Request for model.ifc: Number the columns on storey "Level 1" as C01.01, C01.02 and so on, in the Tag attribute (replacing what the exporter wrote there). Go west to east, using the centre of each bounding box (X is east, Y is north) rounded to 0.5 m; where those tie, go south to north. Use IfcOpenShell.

First a look at what the model holds.

```python
import ifcopenshell
import ifcopenshell.util.element
import ifcopenshell.util.placement

model = ifcopenshell.open("model.ifc")
print(model.schema)
storey = next(s for s in model.by_type("IfcBuildingStorey") if s.Name == "Level 1")
columns = [e for e in ifcopenshell.util.element.get_decomposition(storey) if e.is_a("IfcColumn")]
for e in sorted(columns, key=lambda e: e.id()):
    origin = ifcopenshell.util.placement.get_local_placement(e.ObjectPlacement)[:3, 3]
    print(e.id(), e.Tag, e.Name, origin.round(2) + 0.0, sep=" | ")
```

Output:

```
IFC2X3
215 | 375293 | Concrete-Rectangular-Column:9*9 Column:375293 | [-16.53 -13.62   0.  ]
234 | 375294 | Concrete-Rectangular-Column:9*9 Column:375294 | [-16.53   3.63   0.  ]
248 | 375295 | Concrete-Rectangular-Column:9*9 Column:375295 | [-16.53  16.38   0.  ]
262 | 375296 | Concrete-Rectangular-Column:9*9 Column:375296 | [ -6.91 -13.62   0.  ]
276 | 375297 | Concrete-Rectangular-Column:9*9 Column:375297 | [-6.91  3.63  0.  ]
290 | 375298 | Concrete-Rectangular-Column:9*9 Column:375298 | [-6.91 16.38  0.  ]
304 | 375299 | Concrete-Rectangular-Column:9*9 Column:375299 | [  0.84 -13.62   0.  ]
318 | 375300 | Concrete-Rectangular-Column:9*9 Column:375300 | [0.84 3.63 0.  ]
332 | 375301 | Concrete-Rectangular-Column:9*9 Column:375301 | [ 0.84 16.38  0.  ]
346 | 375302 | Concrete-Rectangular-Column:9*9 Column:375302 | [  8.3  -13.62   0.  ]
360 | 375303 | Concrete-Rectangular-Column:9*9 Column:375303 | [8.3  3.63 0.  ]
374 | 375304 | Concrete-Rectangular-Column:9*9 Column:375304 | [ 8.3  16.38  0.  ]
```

```python
import ifcopenshell
import ifcopenshell.geom
import ifcopenshell.util.element
import ifcopenshell.util.shape

model = ifcopenshell.open("model.ifc")
settings = ifcopenshell.geom.settings()
settings.set("use-world-coords", True)


def centre(element):
    shape = ifcopenshell.geom.create_shape(settings, element)
    return ifcopenshell.util.shape.get_bbox_centroid(shape.geometry)


storey = next(s for s in model.by_type("IfcBuildingStorey") if s.Name == "Level 1")
columns = [e for e in ifcopenshell.util.element.get_decomposition(storey) if e.is_a("IfcColumn")]

# Insertion points can sit at a corner or the storey origin, so sort by the geometry (in metres).
centres = {e: centre(e) for e in columns}
columns.sort(key=lambda e: (round(centres[e][0] / 0.5), centres[e][1]))

for i, e in enumerate(columns, start=1):
    number = f"C01.{i:02d}"
    e.Tag = number
    print(e.id(), number)

model.write("model_rev.ifc")
```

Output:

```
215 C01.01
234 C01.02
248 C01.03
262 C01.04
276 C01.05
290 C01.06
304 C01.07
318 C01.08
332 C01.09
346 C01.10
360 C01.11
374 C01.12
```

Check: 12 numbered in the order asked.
